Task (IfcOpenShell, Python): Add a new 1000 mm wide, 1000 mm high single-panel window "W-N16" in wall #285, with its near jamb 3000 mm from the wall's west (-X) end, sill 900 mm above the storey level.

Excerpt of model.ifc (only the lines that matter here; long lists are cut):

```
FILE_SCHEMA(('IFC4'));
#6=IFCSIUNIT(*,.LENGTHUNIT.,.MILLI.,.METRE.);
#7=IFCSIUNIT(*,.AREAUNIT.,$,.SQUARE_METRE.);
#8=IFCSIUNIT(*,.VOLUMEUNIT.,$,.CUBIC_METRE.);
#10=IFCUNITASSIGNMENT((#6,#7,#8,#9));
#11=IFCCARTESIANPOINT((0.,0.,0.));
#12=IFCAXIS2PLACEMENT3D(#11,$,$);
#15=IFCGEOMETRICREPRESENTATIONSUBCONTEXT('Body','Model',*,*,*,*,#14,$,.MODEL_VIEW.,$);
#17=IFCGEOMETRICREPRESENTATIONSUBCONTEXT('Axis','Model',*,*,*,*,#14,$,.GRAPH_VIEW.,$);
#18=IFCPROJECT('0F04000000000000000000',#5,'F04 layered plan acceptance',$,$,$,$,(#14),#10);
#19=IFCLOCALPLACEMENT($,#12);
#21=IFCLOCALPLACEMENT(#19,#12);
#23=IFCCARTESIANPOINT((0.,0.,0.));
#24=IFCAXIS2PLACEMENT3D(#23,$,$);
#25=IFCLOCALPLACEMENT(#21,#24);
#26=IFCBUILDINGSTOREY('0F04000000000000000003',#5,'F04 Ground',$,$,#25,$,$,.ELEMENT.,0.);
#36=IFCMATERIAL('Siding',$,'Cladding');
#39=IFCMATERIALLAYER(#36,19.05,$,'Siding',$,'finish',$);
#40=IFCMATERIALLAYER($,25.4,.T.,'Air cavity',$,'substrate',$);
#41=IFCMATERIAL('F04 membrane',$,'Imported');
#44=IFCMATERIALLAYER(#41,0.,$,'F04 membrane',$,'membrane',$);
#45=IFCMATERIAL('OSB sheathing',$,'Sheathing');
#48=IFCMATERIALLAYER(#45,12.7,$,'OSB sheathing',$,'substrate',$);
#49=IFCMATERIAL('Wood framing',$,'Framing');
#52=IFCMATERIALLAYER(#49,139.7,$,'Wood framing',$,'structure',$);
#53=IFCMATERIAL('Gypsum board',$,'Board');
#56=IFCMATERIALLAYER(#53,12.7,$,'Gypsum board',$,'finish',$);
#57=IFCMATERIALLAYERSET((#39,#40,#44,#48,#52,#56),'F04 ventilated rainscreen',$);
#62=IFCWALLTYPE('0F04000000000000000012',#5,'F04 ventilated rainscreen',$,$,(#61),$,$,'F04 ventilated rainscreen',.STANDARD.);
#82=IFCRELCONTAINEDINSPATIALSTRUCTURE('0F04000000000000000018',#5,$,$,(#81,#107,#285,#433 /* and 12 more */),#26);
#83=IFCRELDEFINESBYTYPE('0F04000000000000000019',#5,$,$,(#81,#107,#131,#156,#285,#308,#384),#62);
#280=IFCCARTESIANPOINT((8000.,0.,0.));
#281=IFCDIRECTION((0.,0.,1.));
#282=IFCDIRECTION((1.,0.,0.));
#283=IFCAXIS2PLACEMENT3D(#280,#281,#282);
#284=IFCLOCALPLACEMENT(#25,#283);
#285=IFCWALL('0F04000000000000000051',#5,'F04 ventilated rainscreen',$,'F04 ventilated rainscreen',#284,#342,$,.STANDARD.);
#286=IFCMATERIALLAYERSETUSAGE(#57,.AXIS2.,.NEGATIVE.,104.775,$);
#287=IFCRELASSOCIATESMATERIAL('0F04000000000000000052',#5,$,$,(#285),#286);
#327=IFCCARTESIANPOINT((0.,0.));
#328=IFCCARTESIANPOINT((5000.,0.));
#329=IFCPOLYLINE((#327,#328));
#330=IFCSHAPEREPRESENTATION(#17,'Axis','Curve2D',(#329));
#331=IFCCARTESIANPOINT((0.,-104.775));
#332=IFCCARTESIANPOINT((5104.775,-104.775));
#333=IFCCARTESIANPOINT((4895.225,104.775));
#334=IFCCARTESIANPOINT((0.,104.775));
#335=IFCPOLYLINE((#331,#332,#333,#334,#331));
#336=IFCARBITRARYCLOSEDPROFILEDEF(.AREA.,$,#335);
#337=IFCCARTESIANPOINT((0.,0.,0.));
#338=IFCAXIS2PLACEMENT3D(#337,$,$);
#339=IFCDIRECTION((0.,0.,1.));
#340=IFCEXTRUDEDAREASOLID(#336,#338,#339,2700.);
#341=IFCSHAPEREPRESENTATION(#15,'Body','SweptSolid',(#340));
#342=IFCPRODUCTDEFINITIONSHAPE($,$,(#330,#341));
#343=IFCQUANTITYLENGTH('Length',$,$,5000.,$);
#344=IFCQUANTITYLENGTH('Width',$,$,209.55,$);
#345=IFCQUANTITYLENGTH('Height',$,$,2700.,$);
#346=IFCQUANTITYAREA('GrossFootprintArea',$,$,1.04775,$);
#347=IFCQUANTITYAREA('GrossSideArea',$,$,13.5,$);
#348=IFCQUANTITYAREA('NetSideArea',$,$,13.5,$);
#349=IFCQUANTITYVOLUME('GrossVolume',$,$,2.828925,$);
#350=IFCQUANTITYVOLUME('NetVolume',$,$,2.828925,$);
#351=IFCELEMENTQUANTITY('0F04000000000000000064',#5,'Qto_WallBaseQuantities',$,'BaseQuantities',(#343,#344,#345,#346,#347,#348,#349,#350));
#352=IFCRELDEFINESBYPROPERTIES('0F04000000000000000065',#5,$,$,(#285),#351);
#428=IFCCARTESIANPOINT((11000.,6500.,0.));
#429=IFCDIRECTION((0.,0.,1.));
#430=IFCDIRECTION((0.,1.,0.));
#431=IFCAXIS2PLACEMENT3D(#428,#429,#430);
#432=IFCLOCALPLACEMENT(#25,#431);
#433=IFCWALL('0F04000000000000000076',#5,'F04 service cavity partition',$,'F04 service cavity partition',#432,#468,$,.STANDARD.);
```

```python
import numpy as np
import ifcopenshell
import ifcopenshell.api.feature
import ifcopenshell.api.geometry
import ifcopenshell.api.pset
import ifcopenshell.api.root
import ifcopenshell.api.spatial
import ifcopenshell.geom
import ifcopenshell.util.element
import ifcopenshell.util.placement
import ifcopenshell.util.representation
import ifcopenshell.util.shape
import ifcopenshell.util.unit

model = ifcopenshell.open("model.ifc")
unit_scale = ifcopenshell.util.unit.calculate_unit_scale(model)
area_scale = ifcopenshell.util.unit.calculate_unit_scale(model, "AREAUNIT")
volume_scale = ifcopenshell.util.unit.calculate_unit_scale(model, "VOLUMEUNIT")
settings = ifcopenshell.geom.settings()


def volume(element):
    """Net volume in cubic metres, openings subtracted."""
    shape = ifcopenshell.geom.create_shape(settings, element)
    return ifcopenshell.util.shape.get_volume(shape.geometry)


wall = model.by_id(285)
storey = ifcopenshell.util.element.get_container(wall, ifc_class="IfcBuildingStorey")
context = ifcopenshell.util.representation.get_context(model, "Model", "Body", "MODEL_VIEW")
before = volume(wall)

width, height, from_end, sill = 1, 1, 3, 0.9  # metres

# The wall runs along its own X axis, and the end named is its -X end.
wall_shape = ifcopenshell.geom.create_shape(settings, wall)
x, y, z = ifcopenshell.util.shape.get_vertices(wall_shape.geometry).T
start = x.min() + from_end
face, thickness = float(y.min()), float(y.max() - y.min())
wall_matrix = ifcopenshell.util.placement.get_local_placement(wall.ObjectPlacement)
level = ifcopenshell.util.placement.get_local_placement(storey.ObjectPlacement)[2, 3]


def in_wall(x, y):
    """Placement at x, y metres in the wall's axes, at sill height."""
    matrix = wall_matrix.copy()
    matrix[:, 3] = wall_matrix @ np.array([x / unit_scale, y / unit_scale, 0.0, 1.0])
    matrix[2, 3] = level + sill / unit_scale
    return matrix


# Opening: a box that overshoots both wall faces by 50 mm.
opening = ifcopenshell.api.root.create_entity(model, ifc_class="IfcOpeningElement", predefined_type="OPENING")
box = ifcopenshell.api.geometry.add_wall_representation(
    model, context=context, length=width, height=height, thickness=thickness + 0.1
)
ifcopenshell.api.geometry.assign_representation(model, product=opening, representation=box)
ifcopenshell.api.geometry.edit_object_placement(model, product=opening, matrix=in_wall(start, face - 0.05), is_si=False)
ifcopenshell.api.feature.add_feature(model, feature=opening, element=wall)

window = ifcopenshell.api.root.create_entity(model, ifc_class="IfcWindow", name="W-N16", predefined_type="WINDOW")
window.OverallWidth, window.OverallHeight = width / unit_scale, height / unit_scale
window.PartitioningType = "SINGLE_PANEL"
body = ifcopenshell.api.geometry.add_window_representation(
    model,
    context=context,
    overall_width=window.OverallWidth,
    overall_height=window.OverallHeight,
    partition_type="SINGLE_PANEL",
)
ifcopenshell.api.geometry.assign_representation(model, product=window, representation=body)
ifcopenshell.api.spatial.assign_container(model, products=[window], relating_structure=storey)
ifcopenshell.api.feature.add_filling(model, opening=opening, element=window)

# Centre the window in the wall's thickness.
ifcopenshell.api.geometry.edit_object_placement(model, product=window, matrix=in_wall(start, face), is_si=False)
window_shape = ifcopenshell.geom.create_shape(settings, window)
depth = ifcopenshell.util.shape.get_vertices(window_shape.geometry)[:, 1]
offset = face + thickness / 2 - (depth.min() + depth.max()) / 2
ifcopenshell.api.geometry.edit_object_placement(model, product=window, matrix=in_wall(start, offset), is_si=False)

after = volume(wall)

# Update the wall's stored quantities.
qto = model.by_id(ifcopenshell.util.element.get_pset(wall, "Qto_WallBaseQuantities", should_inherit=False)["id"])
ifcopenshell.api.pset.edit_qto(model, qto=qto, properties={
    "NetSideArea": after / thickness / area_scale,
    "NetVolume": after / volume_scale,
})

print(f"wall volume {before:.3f} -> {after:.3f} m3")

model.write("model_updated.ifc")
```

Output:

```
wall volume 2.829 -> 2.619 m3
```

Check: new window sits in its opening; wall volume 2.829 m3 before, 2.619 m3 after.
